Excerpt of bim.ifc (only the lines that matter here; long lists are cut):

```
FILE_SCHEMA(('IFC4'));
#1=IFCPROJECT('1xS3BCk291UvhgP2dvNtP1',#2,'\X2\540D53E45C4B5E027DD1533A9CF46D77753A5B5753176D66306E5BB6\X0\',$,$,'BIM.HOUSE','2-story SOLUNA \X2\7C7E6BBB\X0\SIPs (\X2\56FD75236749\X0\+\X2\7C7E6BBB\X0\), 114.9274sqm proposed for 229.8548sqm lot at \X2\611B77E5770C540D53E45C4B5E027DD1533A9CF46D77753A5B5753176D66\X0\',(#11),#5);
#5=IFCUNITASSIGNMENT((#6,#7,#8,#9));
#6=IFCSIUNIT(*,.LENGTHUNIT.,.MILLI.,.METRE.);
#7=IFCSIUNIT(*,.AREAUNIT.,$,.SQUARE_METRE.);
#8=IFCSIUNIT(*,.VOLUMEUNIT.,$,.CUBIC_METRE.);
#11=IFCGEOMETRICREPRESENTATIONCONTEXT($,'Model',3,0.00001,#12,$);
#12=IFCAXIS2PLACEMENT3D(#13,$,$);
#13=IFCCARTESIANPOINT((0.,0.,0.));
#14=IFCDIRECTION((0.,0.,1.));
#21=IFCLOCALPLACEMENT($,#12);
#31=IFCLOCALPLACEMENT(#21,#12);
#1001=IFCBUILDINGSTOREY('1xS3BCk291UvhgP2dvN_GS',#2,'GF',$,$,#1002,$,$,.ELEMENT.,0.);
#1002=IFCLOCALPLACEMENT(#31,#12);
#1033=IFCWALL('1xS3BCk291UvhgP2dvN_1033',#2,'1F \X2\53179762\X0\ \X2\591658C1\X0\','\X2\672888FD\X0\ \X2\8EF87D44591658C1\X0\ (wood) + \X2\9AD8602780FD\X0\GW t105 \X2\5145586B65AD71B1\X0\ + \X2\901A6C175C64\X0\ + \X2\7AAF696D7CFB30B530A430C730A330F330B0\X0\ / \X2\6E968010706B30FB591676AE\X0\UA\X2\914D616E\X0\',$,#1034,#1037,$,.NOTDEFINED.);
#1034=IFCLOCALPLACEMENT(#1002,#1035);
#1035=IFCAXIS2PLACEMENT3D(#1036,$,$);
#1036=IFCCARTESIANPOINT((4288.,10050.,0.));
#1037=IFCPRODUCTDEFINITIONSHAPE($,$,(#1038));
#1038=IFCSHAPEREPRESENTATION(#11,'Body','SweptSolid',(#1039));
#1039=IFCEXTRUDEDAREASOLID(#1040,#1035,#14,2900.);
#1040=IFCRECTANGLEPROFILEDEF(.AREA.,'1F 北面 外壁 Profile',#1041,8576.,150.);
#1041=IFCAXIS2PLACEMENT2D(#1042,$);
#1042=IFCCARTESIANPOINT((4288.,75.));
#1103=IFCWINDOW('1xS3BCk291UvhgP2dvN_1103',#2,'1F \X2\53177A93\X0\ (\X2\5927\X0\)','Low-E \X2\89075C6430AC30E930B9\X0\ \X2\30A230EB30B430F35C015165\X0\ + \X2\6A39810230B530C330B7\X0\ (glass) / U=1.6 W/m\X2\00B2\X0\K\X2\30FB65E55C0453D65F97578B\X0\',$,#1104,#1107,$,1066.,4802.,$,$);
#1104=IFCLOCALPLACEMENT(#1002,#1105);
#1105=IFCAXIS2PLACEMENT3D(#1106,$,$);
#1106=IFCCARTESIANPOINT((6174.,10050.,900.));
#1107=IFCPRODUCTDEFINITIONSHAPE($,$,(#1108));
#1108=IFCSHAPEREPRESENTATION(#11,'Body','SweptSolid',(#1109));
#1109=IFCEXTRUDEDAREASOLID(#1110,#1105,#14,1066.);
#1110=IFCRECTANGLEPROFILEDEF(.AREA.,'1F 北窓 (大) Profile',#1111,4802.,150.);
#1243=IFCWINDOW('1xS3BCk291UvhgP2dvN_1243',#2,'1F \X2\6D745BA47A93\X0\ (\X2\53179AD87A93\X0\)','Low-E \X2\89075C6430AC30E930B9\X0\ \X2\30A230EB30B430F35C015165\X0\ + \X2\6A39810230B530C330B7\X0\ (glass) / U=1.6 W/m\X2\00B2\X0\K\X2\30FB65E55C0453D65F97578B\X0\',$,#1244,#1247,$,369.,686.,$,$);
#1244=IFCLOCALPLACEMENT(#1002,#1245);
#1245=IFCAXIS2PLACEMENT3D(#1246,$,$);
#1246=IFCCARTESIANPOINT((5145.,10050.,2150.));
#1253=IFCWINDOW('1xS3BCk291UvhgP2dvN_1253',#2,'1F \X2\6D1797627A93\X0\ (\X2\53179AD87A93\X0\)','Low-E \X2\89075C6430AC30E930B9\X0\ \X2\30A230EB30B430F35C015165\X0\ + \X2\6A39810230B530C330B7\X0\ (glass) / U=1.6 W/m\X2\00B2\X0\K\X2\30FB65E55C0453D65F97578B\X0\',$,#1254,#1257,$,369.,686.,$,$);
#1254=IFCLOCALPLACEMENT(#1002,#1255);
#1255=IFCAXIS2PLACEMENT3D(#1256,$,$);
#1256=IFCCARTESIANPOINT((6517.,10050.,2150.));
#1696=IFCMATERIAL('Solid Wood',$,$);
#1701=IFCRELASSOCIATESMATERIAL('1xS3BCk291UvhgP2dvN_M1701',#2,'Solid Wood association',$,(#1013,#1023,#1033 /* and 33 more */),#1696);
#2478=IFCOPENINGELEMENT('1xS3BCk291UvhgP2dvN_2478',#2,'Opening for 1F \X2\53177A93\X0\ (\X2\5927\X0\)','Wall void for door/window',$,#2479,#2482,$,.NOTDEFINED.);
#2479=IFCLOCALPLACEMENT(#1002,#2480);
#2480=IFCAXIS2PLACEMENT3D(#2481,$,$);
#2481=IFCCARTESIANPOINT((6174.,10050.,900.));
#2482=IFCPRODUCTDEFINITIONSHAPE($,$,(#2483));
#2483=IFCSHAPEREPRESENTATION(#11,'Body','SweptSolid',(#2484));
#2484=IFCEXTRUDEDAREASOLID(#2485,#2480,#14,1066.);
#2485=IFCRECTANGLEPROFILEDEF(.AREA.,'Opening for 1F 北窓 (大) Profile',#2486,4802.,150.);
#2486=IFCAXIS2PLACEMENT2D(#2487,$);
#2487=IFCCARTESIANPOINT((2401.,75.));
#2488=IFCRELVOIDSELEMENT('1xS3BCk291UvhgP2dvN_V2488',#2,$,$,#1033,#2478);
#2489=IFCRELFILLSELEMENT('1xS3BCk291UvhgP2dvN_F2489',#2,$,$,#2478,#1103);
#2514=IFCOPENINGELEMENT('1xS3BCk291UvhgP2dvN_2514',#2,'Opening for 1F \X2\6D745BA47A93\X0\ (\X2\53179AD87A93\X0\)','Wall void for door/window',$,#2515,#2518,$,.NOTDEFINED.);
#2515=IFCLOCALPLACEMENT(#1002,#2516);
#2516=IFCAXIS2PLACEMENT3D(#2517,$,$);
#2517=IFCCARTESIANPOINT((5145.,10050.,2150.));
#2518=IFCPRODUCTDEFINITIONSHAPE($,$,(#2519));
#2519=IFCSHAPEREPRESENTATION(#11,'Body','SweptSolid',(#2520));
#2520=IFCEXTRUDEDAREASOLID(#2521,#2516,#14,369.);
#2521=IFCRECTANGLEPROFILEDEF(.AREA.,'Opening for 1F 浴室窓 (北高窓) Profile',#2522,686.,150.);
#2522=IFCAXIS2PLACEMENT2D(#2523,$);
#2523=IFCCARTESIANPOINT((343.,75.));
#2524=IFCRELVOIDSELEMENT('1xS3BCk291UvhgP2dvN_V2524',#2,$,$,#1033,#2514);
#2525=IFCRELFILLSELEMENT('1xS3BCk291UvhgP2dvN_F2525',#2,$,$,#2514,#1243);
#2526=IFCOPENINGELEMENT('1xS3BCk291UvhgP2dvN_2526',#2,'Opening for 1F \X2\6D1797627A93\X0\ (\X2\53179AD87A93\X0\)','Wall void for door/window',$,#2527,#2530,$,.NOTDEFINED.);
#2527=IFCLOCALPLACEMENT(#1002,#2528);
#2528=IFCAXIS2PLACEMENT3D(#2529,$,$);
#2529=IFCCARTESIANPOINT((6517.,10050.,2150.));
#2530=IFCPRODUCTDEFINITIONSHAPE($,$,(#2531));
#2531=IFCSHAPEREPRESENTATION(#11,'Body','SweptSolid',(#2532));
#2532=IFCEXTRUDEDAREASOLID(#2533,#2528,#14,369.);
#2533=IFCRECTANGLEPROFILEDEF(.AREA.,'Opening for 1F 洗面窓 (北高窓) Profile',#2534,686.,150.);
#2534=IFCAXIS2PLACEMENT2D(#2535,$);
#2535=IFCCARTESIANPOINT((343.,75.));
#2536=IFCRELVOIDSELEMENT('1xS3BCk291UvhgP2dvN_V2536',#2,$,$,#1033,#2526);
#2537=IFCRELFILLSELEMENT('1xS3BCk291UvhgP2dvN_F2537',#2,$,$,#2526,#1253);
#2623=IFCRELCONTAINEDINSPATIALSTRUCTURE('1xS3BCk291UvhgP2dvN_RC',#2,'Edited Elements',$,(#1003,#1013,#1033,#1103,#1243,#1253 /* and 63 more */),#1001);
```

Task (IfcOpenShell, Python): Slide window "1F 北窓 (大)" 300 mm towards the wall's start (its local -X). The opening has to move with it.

```python
import ifcopenshell
import ifcopenshell.api.geometry
import ifcopenshell.util.placement

model = ifcopenshell.open("bim.ifc")

window = model.by_guid("1xS3BCk291UvhgP2dvN_1103")
opening = window.FillsVoids[0].RelatingOpeningElement
wall = opening.VoidsElements[0].RelatingBuildingElement

wall_matrix = ifcopenshell.util.placement.get_local_placement(wall.ObjectPlacement)
shift = wall_matrix[:3, 0] * -300.0
before = ifcopenshell.util.placement.get_local_placement(window.ObjectPlacement)[:3, 3].copy()

# The window is not placed relative to its opening, so move both.
for product in (opening, window):
    matrix = ifcopenshell.util.placement.get_local_placement(product.ObjectPlacement)
    matrix[:3, 3] += shift
    ifcopenshell.api.geometry.edit_object_placement(model, product=product, matrix=matrix, is_si=False)

after = ifcopenshell.util.placement.get_local_placement(window.ObjectPlacement)[:3, 3]
print("window moved by", (after - before).round(3) + 0.0)

model.write("bim_rev.ifc")
```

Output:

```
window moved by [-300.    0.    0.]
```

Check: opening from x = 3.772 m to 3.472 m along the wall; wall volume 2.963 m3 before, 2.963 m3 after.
